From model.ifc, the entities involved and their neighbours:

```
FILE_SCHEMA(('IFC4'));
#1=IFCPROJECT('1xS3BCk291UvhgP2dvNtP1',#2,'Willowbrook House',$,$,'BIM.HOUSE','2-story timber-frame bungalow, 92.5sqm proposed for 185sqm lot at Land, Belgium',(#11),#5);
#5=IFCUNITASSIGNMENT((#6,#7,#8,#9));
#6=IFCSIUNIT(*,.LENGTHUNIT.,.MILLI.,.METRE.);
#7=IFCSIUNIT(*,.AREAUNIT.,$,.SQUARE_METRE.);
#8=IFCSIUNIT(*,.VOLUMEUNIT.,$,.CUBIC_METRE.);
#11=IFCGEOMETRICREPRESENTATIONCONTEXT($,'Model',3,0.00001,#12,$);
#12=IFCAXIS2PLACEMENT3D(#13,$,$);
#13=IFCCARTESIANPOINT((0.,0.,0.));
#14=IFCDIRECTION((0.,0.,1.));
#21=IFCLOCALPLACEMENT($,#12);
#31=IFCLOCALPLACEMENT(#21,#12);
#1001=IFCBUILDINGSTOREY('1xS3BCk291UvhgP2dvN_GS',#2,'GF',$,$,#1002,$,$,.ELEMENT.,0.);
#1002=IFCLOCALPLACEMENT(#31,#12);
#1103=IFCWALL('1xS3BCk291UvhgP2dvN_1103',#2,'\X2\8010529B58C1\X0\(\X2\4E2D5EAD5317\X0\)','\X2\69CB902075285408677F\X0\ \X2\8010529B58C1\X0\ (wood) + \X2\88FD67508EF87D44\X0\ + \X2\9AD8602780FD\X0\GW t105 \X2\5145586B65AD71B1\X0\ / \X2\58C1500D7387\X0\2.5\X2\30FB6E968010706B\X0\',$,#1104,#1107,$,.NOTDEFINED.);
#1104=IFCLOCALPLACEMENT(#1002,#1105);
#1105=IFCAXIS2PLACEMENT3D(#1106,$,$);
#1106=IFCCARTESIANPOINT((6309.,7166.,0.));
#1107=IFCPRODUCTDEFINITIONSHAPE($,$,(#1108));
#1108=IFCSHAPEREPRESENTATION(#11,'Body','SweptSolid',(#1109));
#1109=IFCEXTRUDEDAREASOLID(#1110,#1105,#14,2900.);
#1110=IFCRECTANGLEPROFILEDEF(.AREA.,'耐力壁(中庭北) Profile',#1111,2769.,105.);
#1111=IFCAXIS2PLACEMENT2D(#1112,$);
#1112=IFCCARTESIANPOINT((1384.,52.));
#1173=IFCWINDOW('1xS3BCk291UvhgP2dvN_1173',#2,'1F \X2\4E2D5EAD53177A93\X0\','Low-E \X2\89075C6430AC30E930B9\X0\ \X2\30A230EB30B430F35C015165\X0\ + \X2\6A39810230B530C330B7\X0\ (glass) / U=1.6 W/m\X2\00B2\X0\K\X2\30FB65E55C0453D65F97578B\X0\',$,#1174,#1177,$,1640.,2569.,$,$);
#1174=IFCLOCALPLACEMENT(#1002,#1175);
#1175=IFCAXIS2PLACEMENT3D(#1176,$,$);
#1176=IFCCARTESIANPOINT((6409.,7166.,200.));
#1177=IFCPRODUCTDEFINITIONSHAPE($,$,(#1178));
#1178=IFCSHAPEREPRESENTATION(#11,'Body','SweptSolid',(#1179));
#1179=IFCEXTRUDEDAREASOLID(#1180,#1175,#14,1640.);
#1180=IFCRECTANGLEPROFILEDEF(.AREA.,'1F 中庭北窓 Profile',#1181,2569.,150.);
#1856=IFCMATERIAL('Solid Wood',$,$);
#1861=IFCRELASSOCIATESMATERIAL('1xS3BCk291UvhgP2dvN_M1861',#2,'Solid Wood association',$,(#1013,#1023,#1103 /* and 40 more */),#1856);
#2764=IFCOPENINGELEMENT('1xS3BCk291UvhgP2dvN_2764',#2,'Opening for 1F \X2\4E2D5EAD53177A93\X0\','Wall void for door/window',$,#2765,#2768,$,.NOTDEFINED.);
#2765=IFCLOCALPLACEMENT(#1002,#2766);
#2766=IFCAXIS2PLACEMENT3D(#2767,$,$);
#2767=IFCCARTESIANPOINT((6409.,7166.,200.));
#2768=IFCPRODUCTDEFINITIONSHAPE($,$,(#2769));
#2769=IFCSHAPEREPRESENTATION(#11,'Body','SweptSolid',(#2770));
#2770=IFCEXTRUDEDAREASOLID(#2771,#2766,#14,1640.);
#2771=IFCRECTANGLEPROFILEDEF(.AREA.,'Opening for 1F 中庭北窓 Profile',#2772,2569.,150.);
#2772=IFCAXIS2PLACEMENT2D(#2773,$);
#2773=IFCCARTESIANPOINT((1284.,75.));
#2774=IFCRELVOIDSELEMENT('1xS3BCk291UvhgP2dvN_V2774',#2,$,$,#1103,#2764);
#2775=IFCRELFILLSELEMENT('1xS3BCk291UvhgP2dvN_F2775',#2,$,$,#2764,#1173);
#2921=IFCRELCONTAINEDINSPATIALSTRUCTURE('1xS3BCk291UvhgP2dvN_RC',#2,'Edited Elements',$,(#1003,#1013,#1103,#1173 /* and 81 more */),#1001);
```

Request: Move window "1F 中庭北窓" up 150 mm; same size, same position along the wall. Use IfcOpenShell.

```python
import numpy as np
import ifcopenshell
import ifcopenshell.api.geometry
import ifcopenshell.util.placement
import ifcopenshell.util.unit

model = ifcopenshell.open("model.ifc")
unit_scale = ifcopenshell.util.unit.calculate_unit_scale(model)

window = model.by_guid("1xS3BCk291UvhgP2dvN_1173")
opening = window.FillsVoids[0].RelatingOpeningElement
dz = 0.15 / unit_scale

shift = np.array([0.0, 0.0, dz])
# The window is not placed relative to its opening, so move both.
for product in (opening, window):
    matrix = ifcopenshell.util.placement.get_local_placement(product.ObjectPlacement)
    matrix[:3, 3] += shift
    ifcopenshell.api.geometry.edit_object_placement(model, product=product, matrix=matrix, is_si=False)

print(f"moved by {dz * unit_scale:+.3f} m")

model.write("model_v2.ifc")
```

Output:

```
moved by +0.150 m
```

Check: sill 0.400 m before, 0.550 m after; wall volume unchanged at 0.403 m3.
